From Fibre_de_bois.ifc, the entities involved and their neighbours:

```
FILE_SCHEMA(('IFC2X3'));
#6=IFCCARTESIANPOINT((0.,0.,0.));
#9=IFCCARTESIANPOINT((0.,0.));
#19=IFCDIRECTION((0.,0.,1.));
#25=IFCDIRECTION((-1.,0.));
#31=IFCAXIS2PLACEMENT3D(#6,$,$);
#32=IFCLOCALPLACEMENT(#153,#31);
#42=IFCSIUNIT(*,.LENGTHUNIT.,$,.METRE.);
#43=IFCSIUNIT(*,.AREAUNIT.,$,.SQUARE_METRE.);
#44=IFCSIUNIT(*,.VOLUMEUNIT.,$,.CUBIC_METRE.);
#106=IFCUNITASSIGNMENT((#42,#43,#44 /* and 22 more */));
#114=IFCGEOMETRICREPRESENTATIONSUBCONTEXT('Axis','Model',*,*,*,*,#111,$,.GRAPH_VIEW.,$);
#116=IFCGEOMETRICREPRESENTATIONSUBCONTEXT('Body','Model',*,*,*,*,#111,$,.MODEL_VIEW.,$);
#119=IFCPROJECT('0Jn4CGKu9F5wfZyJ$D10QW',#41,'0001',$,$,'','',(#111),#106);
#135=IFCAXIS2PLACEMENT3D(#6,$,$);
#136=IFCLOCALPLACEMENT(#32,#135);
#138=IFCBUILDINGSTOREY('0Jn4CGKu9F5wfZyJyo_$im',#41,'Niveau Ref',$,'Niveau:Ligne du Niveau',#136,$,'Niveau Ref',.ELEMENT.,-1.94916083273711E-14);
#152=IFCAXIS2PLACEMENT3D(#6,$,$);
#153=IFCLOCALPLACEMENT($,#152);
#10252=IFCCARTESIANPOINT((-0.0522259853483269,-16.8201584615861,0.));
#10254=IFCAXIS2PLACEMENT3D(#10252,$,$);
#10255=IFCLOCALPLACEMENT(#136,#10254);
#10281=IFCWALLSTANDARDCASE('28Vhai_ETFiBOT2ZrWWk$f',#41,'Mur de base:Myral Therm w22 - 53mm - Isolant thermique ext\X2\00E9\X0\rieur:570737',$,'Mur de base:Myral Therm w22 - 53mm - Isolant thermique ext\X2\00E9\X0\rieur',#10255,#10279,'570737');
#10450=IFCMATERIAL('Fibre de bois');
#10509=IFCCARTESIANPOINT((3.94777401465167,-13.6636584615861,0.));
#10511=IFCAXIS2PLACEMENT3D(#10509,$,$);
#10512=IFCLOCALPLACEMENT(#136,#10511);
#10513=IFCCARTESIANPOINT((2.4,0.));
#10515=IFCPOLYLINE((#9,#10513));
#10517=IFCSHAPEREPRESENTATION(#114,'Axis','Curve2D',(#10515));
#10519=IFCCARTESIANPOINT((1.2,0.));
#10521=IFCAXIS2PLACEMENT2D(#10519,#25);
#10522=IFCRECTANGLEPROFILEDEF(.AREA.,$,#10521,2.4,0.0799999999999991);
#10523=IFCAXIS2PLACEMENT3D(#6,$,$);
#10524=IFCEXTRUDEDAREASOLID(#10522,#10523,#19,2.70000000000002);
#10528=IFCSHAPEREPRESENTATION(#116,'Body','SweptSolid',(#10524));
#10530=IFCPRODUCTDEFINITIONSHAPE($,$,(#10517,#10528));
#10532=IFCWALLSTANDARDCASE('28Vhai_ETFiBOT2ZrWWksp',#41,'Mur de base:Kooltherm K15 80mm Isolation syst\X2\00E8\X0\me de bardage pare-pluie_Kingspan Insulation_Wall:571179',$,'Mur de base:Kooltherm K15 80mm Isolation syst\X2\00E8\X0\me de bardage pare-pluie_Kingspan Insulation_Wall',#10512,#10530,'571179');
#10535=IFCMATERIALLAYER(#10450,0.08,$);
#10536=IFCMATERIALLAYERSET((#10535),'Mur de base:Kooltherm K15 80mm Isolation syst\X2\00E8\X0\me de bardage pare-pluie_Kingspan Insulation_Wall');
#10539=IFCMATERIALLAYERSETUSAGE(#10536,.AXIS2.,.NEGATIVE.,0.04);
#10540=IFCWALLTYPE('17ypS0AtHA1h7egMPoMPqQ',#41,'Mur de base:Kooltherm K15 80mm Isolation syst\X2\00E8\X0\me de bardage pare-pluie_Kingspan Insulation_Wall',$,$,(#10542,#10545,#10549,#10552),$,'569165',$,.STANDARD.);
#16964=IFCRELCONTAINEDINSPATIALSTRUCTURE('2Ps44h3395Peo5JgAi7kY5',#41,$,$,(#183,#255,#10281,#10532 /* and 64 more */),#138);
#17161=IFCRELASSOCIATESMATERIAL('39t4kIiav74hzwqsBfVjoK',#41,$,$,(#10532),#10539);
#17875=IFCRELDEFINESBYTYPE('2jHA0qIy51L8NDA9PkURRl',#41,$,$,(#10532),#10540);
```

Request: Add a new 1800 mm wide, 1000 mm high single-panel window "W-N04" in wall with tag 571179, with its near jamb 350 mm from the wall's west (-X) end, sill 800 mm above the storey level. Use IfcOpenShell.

```python
import numpy as np
import ifcopenshell
import ifcopenshell.api.feature
import ifcopenshell.api.geometry
import ifcopenshell.api.root
import ifcopenshell.api.spatial
import ifcopenshell.api.type
import ifcopenshell.geom
import ifcopenshell.util.element
import ifcopenshell.util.placement
import ifcopenshell.util.representation
import ifcopenshell.util.shape
import ifcopenshell.util.unit

model = ifcopenshell.open("Fibre_de_bois.ifc")
unit_scale = ifcopenshell.util.unit.calculate_unit_scale(model)
settings = ifcopenshell.geom.settings()


def volume(element):
    """Net volume in cubic metres, openings subtracted."""
    shape = ifcopenshell.geom.create_shape(settings, element)
    return ifcopenshell.util.shape.get_volume(shape.geometry)


wall = model.by_guid("28Vhai_ETFiBOT2ZrWWksp")
storey = ifcopenshell.util.element.get_container(wall, ifc_class="IfcBuildingStorey")
context = ifcopenshell.util.representation.get_context(model, "Model", "Body", "MODEL_VIEW")
before = volume(wall)

width, height, from_end, sill = 1.8, 1, 0.35, 0.8  # metres

# The wall runs along its own X axis, and the end named is its -X end.
wall_shape = ifcopenshell.geom.create_shape(settings, wall)
x, y, z = ifcopenshell.util.shape.get_vertices(wall_shape.geometry).T
start = x.min() + from_end
face, thickness = float(y.min()), float(y.max() - y.min())
wall_matrix = ifcopenshell.util.placement.get_local_placement(wall.ObjectPlacement)
level = ifcopenshell.util.placement.get_local_placement(storey.ObjectPlacement)[2, 3]


def in_wall(x, y):
    """Placement at x, y metres in the wall's axes, at sill height."""
    matrix = wall_matrix.copy()
    matrix[:, 3] = wall_matrix @ np.array([x / unit_scale, y / unit_scale, 0.0, 1.0])
    matrix[2, 3] = level + sill / unit_scale
    return matrix


# Opening: a box that overshoots both wall faces by 50 mm.
opening = ifcopenshell.api.root.create_entity(model, ifc_class="IfcOpeningElement")
box = ifcopenshell.api.geometry.add_wall_representation(
    model, context=context, length=width, height=height, thickness=thickness + 0.1
)
ifcopenshell.api.geometry.assign_representation(model, product=opening, representation=box)
ifcopenshell.api.geometry.edit_object_placement(model, product=opening, matrix=in_wall(start, face - 0.05), is_si=False)
ifcopenshell.api.feature.add_feature(model, feature=opening, element=wall)

window = ifcopenshell.api.root.create_entity(model, ifc_class="IfcWindow", name="W-N04")
window.OverallWidth, window.OverallHeight = width / unit_scale, height / unit_scale
body = ifcopenshell.api.geometry.add_window_representation(
    model,
    context=context,
    overall_width=window.OverallWidth,
    overall_height=window.OverallHeight,
    partition_type="SINGLE_PANEL",
)
ifcopenshell.api.geometry.assign_representation(model, product=window, representation=body)
ifcopenshell.api.spatial.assign_container(model, products=[window], relating_structure=storey)
fills = ifcopenshell.api.feature.add_filling(model, opening=opening, element=window)
fills.OwnerHistory = window.OwnerHistory  # required in IFC2X3

# IFC2X3 keeps the operation on the window style.
style = ifcopenshell.api.root.create_entity(model, ifc_class="IfcWindowStyle", name="W-N04")
style.OperationType, style.ConstructionType = "SINGLE_PANEL", "NOTDEFINED"
style.ParameterTakesPrecedence = style.Sizeable = False
ifcopenshell.api.type.assign_type(model, related_objects=[window], relating_type=style)

# Centre the window in the wall's thickness.
ifcopenshell.api.geometry.edit_object_placement(model, product=window, matrix=in_wall(start, face), is_si=False)
window_shape = ifcopenshell.geom.create_shape(settings, window)
depth = ifcopenshell.util.shape.get_vertices(window_shape.geometry)[:, 1]
offset = face + thickness / 2 - (depth.min() + depth.max()) / 2
ifcopenshell.api.geometry.edit_object_placement(model, product=window, matrix=in_wall(start, offset), is_si=False)

after = volume(wall)

print(f"wall volume {before:.3f} -> {after:.3f} m3")

model.write("Fibre_de_bois_rev.ifc")
```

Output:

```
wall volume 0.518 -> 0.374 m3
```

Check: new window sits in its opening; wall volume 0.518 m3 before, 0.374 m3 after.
